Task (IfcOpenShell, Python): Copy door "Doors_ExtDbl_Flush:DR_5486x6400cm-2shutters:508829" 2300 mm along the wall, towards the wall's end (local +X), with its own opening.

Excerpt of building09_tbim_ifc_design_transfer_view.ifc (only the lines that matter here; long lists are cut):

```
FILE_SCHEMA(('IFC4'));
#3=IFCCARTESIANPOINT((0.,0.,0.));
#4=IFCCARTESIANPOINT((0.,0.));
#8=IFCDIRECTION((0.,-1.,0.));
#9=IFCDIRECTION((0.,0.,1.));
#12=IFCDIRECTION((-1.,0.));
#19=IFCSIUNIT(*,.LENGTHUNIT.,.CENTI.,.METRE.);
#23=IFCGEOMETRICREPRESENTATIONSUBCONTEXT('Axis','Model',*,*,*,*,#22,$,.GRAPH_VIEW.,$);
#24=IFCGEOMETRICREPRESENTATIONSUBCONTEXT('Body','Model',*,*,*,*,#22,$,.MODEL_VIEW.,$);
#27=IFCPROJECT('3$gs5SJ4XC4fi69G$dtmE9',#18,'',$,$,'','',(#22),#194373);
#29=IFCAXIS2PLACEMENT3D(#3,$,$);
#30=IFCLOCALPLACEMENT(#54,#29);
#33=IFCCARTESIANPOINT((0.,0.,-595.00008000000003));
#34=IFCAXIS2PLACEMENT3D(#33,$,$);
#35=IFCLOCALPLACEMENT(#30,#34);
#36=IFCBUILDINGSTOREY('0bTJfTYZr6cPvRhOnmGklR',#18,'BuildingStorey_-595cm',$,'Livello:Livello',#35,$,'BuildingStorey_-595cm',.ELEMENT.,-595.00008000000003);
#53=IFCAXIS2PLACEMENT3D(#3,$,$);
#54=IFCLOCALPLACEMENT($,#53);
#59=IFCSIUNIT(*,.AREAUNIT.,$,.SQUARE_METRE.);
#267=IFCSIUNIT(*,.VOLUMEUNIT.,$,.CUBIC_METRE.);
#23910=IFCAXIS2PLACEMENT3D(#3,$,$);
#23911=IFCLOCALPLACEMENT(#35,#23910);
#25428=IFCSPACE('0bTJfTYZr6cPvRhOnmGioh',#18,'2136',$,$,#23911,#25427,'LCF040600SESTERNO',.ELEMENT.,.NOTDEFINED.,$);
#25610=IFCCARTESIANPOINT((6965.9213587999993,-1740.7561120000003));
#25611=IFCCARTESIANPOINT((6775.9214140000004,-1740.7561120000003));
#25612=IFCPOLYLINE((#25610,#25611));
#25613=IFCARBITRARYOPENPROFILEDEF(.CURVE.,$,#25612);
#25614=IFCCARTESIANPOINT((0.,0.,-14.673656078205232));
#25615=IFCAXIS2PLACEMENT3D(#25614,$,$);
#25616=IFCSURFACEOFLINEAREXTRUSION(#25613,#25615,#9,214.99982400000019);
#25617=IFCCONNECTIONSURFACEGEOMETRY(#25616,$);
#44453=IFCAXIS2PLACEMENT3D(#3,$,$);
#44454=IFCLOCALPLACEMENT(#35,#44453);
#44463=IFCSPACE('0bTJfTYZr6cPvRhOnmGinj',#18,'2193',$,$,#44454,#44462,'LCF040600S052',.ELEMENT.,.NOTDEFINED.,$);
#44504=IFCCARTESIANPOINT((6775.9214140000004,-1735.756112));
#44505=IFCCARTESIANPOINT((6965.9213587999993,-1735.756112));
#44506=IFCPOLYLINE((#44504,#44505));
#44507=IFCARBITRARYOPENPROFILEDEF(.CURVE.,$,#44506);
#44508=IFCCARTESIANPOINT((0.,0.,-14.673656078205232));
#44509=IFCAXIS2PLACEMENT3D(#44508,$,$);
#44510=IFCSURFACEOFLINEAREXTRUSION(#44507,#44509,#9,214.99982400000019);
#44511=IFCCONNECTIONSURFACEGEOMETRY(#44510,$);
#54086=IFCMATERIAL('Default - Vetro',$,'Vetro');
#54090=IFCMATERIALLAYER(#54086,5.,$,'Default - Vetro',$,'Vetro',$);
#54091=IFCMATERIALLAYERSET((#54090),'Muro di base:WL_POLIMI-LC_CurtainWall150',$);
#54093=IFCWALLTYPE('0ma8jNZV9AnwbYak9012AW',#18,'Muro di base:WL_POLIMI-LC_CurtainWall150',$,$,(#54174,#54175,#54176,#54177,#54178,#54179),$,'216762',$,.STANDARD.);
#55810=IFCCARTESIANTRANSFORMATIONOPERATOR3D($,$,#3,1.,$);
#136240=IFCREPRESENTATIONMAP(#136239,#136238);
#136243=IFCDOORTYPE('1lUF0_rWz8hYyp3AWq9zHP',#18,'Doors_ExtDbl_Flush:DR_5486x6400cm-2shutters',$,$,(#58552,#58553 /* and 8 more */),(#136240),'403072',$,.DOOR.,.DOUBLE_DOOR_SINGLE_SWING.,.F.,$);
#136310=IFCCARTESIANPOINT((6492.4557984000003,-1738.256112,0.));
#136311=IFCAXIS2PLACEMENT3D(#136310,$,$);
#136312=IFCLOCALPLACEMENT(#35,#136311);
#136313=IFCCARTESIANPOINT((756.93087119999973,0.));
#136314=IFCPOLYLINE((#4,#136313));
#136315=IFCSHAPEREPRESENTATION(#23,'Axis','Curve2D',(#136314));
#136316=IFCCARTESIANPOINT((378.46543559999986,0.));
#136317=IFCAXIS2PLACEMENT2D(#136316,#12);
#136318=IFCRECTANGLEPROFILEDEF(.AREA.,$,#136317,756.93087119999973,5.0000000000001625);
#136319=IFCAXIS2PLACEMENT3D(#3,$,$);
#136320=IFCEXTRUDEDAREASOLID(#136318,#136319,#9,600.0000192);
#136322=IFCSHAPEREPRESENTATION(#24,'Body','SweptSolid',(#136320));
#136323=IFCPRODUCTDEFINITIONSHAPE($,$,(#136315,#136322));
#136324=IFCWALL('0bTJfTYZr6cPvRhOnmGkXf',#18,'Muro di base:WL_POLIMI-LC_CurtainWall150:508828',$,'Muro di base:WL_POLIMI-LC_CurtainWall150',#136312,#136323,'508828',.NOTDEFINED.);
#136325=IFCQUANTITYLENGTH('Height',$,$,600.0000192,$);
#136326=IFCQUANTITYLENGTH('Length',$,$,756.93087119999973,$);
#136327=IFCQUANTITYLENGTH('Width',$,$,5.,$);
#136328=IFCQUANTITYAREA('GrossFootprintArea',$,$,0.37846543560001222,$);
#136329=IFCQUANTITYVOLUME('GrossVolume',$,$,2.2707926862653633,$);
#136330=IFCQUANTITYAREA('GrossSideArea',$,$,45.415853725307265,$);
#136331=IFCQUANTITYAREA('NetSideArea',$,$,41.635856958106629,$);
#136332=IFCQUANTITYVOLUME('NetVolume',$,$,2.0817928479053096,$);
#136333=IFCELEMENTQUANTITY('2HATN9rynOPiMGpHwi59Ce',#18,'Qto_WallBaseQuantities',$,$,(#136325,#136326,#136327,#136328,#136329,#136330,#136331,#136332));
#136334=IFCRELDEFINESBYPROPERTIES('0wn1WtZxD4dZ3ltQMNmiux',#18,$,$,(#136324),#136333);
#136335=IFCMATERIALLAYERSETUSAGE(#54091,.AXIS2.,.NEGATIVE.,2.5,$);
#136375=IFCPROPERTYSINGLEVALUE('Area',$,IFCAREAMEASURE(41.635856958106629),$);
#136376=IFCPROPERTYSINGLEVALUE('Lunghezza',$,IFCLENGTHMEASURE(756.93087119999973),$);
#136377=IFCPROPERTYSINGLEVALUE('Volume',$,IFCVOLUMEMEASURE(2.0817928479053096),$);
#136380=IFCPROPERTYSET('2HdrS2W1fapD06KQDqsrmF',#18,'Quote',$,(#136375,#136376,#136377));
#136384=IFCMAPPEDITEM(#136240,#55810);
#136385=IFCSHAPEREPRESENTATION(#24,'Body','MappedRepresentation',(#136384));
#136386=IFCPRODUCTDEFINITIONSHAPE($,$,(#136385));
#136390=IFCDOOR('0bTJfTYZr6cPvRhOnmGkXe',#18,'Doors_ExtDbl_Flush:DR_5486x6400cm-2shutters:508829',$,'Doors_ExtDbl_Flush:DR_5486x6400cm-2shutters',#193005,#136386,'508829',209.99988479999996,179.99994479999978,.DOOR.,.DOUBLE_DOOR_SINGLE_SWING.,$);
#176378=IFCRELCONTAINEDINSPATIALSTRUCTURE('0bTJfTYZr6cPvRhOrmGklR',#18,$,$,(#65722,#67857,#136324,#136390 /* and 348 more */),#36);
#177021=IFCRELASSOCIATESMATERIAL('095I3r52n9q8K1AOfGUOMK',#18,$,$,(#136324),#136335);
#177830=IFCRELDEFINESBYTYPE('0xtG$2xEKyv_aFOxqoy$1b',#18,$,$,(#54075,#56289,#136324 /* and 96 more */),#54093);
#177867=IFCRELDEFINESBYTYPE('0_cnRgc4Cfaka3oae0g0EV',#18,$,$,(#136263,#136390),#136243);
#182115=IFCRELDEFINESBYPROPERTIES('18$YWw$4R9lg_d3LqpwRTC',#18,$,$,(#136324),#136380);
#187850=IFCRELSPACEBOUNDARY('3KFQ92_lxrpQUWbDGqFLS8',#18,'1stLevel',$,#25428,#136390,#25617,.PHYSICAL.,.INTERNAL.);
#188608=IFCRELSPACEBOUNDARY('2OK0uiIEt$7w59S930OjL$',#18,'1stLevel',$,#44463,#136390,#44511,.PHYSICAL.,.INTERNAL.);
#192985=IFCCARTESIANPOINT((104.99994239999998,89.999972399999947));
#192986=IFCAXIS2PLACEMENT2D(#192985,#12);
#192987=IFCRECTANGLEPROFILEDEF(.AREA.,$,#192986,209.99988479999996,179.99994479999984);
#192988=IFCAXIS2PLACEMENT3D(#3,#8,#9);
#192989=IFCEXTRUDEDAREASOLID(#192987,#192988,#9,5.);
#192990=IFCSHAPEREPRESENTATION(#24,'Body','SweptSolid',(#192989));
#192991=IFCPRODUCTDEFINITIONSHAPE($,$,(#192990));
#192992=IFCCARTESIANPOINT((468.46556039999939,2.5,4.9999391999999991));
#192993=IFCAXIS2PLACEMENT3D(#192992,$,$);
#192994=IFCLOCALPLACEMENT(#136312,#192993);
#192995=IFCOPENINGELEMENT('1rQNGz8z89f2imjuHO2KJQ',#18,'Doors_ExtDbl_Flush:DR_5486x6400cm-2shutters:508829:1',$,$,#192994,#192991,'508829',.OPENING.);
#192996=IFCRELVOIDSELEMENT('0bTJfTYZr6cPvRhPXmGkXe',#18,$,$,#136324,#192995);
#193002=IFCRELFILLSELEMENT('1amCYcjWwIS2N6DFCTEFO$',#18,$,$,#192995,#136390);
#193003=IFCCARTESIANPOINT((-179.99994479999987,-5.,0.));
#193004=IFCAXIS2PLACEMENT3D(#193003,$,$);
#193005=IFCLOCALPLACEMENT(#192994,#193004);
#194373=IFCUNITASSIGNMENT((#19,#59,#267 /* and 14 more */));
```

```python
import numpy as np
import ifcopenshell
import ifcopenshell.api.feature
import ifcopenshell.api.geometry
import ifcopenshell.api.pset
import ifcopenshell.api.root
import ifcopenshell.geom
import ifcopenshell.util.element
import ifcopenshell.util.placement
import ifcopenshell.util.shape
import ifcopenshell.util.unit

model = ifcopenshell.open("building09_tbim_ifc_design_transfer_view.ifc")
unit_scale = ifcopenshell.util.unit.calculate_unit_scale(model)
area_scale = ifcopenshell.util.unit.calculate_unit_scale(model, "AREAUNIT")
volume_scale = ifcopenshell.util.unit.calculate_unit_scale(model, "VOLUMEUNIT")
settings = ifcopenshell.geom.settings()


def volume(element):
    """Net volume in cubic metres, openings subtracted."""
    shape = ifcopenshell.geom.create_shape(settings, element)
    return ifcopenshell.util.shape.get_volume(shape.geometry)


def reuse_history(source, copy):
    """copy_class also copies each property set's owner history, people and application; keep the originals."""
    for rel in copy.IsDefinedBy:
        if rel.is_a("IfcRelDefinesByProperties") and (history := rel.RelatingPropertyDefinition.OwnerHistory):
            rel.RelatingPropertyDefinition.OwnerHistory = source.OwnerHistory
            ifcopenshell.util.element.remove_deep2(model, history)


door = model.by_guid("0bTJfTYZr6cPvRhOnmGkXe")
opening = door.FillsVoids[0].RelatingOpeningElement
wall = opening.VoidsElements[0].RelatingBuildingElement
before = volume(wall)
shift = ifcopenshell.util.placement.get_local_placement(wall.ObjectPlacement)[:3, 0] * 2.3 / unit_scale

# copy_class copies the void relationship, type, container and properties, but no geometry.
new_opening = ifcopenshell.api.root.copy_class(model, product=opening)
new_opening.Representation = ifcopenshell.util.element.copy_deep(
    model, opening.Representation, exclude=["IfcGeometricRepresentationContext", "IfcRepresentationMap"]
)
new_opening.Name = "Doors_ExtDbl_Flush:DR_5486x6400cm-2shutters"
new_opening.Tag = None
reuse_history(opening, new_opening)
new_door = ifcopenshell.api.root.copy_class(model, product=door)
new_door.Representation = ifcopenshell.util.element.copy_deep(
    model, door.Representation, exclude=["IfcGeometricRepresentationContext", "IfcRepresentationMap"]
)
new_door.Name = "Doors_ExtDbl_Flush:DR_5486x6400cm-2shutters"
new_door.Tag = None
reuse_history(door, new_door)
ifcopenshell.api.feature.add_filling(model, opening=new_opening, element=new_door)

for old, new in ((opening, new_opening), (door, new_door)):
    matrix = ifcopenshell.util.placement.get_local_placement(old.ObjectPlacement)
    matrix[:3, 3] += shift
    ifcopenshell.api.geometry.edit_object_placement(model, product=new, matrix=matrix, is_si=False)

# The copied space boundaries still share their surfaces with the original.
for rel in new_door.ProvidesBoundaries:
    if rel.ConnectionGeometry:
        rel.ConnectionGeometry = ifcopenshell.util.element.copy_deep(model, rel.ConnectionGeometry)

# Space boundary surfaces are stored in each space's coordinates; move them too.
for rel in new_door.ProvidesBoundaries:
    if not rel.ConnectionGeometry:
        continue
    surface = rel.ConnectionGeometry.SurfaceOnRelatingElement
    space_matrix = ifcopenshell.util.placement.get_local_placement(rel.RelatingSpace.ObjectPlacement)
    point = np.array(surface.Position.Location.Coordinates) + space_matrix[:3, :3].T @ shift
    surface.Position = model.createIfcAxis2Placement3D(
        model.createIfcCartesianPoint(point.tolist()), surface.Position.Axis, surface.Position.RefDirection
    )

after = volume(wall)
thickness = 0.05  # wall thickness in metres

# Update the wall's stored quantities.
qto = model.by_id(ifcopenshell.util.element.get_pset(wall, "Qto_WallBaseQuantities", should_inherit=False)["id"])
ifcopenshell.api.pset.edit_qto(model, qto=qto, properties={
    "NetSideArea": after / thickness / area_scale,
    "NetVolume": after / volume_scale,
})
pset = model.by_id(ifcopenshell.util.element.get_pset(wall, "Quote", should_inherit=False)["id"])
ifcopenshell.api.pset.edit_pset(model, pset=pset, properties={
    "Area": model.create_entity("IfcAreaMeasure", after / thickness / area_scale),
    "Volume": model.create_entity("IfcVolumeMeasure", after / volume_scale),
})

print(f"wall volume {before:.3f} -> {after:.3f} m3")

model.write("building09_tbim_ifc_design_transfer_view_edited.ifc")
```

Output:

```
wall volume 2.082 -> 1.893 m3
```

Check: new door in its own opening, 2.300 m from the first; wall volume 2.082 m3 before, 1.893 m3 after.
